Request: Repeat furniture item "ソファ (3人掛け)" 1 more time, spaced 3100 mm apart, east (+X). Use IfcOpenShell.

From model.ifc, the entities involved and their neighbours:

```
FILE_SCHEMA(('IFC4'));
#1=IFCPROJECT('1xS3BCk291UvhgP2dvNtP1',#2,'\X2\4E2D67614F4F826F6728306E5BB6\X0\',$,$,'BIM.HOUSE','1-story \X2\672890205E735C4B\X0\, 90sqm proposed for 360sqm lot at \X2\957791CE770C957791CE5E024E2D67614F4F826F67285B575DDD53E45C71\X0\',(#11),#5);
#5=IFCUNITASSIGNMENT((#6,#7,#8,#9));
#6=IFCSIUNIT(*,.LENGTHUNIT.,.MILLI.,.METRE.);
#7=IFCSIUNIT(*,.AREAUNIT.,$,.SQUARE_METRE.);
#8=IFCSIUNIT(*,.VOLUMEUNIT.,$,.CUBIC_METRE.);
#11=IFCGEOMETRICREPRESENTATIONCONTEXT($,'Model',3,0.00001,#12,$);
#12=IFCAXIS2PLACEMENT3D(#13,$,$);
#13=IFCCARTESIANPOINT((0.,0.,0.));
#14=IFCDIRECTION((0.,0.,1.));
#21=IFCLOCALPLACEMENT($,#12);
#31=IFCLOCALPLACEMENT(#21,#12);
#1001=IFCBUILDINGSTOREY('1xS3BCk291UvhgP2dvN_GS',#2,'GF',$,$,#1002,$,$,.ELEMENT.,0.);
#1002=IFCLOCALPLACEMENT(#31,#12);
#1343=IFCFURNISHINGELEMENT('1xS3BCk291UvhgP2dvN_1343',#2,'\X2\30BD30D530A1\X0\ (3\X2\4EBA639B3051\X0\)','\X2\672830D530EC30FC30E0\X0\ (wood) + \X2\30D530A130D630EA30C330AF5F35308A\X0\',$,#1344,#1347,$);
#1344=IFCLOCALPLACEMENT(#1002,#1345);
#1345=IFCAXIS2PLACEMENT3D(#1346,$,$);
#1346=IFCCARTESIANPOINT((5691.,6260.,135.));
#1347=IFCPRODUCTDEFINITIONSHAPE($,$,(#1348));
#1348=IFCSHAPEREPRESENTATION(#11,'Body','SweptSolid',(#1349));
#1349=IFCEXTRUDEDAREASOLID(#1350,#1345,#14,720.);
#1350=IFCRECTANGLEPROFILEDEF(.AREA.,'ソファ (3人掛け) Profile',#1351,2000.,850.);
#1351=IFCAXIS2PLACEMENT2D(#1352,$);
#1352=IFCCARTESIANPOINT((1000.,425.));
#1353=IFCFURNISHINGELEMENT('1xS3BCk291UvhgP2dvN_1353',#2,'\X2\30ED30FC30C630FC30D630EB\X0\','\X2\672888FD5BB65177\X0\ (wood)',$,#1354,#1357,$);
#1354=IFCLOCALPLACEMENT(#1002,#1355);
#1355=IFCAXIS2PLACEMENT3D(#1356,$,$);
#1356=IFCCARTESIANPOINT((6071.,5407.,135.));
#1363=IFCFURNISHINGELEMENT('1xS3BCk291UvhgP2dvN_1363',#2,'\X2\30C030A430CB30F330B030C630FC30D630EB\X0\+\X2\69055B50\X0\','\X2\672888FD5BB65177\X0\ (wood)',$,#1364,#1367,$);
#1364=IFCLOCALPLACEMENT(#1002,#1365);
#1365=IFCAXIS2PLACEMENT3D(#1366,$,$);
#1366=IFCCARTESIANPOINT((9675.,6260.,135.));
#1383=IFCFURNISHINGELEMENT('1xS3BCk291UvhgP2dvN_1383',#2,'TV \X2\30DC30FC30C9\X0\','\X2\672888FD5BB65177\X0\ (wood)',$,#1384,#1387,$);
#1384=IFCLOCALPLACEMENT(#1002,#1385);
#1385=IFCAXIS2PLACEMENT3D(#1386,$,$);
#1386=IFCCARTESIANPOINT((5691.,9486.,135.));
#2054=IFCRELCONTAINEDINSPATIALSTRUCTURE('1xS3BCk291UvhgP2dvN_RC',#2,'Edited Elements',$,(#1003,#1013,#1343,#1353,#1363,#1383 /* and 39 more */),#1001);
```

```python
import numpy as np
import ifcopenshell
import ifcopenshell.api.geometry
import ifcopenshell.api.root
import ifcopenshell.util.element
import ifcopenshell.util.placement

model = ifcopenshell.open("model.ifc")


def reuse_history(source, copy):
    """copy_class also copies each property set's owner history, people and application; keep the originals."""
    for rel in copy.IsDefinedBy:
        if rel.is_a("IfcRelDefinesByProperties") and (history := rel.RelatingPropertyDefinition.OwnerHistory):
            rel.RelatingPropertyDefinition.OwnerHistory = source.OwnerHistory
            ifcopenshell.util.element.remove_deep2(model, history)


source = model.by_guid("1xS3BCk291UvhgP2dvN_1343")
base = ifcopenshell.util.placement.get_local_placement(source.ObjectPlacement)
step = np.array([1.0, 0.0, 0.0]) * 3100.0

for i in range(1, 2):
    copy = ifcopenshell.api.root.copy_class(model, product=source)
    copy.Representation = ifcopenshell.util.element.copy_deep(
        model, source.Representation, exclude=["IfcGeometricRepresentationContext", "IfcRepresentationMap"]
    )
    reuse_history(source, copy)
    matrix = base.copy()
    matrix[:3, 3] += i * step
    print("added at", matrix[:3, 3].round(3) + 0.0)
    ifcopenshell.api.geometry.edit_object_placement(model, product=copy, matrix=matrix, is_si=False)

model.write("model-out.ifc")
```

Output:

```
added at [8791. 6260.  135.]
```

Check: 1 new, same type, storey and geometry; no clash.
